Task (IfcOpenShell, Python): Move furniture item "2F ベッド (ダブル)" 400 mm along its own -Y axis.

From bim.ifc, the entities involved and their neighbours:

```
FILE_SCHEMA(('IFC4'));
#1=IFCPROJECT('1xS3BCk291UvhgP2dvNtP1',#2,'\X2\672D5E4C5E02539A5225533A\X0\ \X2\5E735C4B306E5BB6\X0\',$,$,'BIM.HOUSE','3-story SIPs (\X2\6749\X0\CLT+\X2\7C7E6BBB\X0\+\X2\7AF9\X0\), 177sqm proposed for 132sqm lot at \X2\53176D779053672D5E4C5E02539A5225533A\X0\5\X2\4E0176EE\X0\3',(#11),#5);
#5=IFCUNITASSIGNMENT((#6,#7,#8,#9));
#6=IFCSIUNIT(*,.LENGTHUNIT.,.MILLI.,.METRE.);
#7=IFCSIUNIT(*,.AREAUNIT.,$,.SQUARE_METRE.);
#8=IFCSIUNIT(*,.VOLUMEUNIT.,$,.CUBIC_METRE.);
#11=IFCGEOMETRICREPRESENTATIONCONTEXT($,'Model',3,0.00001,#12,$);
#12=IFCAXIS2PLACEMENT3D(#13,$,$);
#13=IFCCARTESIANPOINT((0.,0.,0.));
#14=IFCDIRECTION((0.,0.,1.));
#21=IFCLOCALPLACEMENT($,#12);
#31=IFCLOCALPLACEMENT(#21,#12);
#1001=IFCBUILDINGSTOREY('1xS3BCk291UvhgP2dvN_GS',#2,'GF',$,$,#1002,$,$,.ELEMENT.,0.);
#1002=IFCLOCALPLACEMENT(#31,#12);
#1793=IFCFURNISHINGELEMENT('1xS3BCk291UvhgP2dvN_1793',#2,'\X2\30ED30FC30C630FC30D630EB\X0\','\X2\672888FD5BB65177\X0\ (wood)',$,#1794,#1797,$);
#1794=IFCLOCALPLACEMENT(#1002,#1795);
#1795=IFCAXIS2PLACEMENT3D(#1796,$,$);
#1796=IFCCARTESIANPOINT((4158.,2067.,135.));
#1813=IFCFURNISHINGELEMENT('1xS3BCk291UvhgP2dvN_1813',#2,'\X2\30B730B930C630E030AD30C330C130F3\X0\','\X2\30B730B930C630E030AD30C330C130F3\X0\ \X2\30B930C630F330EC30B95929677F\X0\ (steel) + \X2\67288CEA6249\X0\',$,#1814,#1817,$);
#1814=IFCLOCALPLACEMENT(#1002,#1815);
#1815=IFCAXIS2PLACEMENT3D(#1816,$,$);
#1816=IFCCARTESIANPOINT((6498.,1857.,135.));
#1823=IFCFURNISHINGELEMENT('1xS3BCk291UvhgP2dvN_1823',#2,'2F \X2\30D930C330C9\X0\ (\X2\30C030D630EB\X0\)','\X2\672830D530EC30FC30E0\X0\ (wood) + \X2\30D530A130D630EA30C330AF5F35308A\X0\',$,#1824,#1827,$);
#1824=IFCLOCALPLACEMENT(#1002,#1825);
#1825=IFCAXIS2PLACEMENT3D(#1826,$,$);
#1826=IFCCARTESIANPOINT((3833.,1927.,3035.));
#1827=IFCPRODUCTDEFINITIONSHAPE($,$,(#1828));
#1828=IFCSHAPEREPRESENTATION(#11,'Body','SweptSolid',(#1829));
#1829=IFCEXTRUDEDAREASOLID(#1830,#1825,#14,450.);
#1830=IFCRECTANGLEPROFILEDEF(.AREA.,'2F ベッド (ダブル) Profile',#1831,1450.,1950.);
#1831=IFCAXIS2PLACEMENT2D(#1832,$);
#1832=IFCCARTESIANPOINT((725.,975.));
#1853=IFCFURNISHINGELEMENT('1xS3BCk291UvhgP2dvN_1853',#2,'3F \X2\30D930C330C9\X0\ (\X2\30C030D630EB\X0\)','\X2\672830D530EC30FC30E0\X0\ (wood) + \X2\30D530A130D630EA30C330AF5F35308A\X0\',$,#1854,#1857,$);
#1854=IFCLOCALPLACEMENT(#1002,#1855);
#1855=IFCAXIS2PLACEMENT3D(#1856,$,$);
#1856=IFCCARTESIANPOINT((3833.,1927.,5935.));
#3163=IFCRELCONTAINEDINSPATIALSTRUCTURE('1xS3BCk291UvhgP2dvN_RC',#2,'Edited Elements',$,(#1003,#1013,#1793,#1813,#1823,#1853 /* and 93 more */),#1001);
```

```python
import ifcopenshell
import ifcopenshell.api.geometry
import ifcopenshell.util.placement
import ifcopenshell.util.unit

model = ifcopenshell.open("bim.ifc")
unit_scale = ifcopenshell.util.unit.calculate_unit_scale(model)

item = model.by_id(1823)
matrix = ifcopenshell.util.placement.get_local_placement(item.ObjectPlacement)
matrix[:3, 3] -= matrix[:3, 1] * 0.4 / unit_scale
ifcopenshell.api.geometry.edit_object_placement(model, product=item, matrix=matrix, is_si=False)

print(ifcopenshell.util.placement.get_local_placement(item.ObjectPlacement).round(3) + 0.0)

model.write("bim_v2.ifc")
```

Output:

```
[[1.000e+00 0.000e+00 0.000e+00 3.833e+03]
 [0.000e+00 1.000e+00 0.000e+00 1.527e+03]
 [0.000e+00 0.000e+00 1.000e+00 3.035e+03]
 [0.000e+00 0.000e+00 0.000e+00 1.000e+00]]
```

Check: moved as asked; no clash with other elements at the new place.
